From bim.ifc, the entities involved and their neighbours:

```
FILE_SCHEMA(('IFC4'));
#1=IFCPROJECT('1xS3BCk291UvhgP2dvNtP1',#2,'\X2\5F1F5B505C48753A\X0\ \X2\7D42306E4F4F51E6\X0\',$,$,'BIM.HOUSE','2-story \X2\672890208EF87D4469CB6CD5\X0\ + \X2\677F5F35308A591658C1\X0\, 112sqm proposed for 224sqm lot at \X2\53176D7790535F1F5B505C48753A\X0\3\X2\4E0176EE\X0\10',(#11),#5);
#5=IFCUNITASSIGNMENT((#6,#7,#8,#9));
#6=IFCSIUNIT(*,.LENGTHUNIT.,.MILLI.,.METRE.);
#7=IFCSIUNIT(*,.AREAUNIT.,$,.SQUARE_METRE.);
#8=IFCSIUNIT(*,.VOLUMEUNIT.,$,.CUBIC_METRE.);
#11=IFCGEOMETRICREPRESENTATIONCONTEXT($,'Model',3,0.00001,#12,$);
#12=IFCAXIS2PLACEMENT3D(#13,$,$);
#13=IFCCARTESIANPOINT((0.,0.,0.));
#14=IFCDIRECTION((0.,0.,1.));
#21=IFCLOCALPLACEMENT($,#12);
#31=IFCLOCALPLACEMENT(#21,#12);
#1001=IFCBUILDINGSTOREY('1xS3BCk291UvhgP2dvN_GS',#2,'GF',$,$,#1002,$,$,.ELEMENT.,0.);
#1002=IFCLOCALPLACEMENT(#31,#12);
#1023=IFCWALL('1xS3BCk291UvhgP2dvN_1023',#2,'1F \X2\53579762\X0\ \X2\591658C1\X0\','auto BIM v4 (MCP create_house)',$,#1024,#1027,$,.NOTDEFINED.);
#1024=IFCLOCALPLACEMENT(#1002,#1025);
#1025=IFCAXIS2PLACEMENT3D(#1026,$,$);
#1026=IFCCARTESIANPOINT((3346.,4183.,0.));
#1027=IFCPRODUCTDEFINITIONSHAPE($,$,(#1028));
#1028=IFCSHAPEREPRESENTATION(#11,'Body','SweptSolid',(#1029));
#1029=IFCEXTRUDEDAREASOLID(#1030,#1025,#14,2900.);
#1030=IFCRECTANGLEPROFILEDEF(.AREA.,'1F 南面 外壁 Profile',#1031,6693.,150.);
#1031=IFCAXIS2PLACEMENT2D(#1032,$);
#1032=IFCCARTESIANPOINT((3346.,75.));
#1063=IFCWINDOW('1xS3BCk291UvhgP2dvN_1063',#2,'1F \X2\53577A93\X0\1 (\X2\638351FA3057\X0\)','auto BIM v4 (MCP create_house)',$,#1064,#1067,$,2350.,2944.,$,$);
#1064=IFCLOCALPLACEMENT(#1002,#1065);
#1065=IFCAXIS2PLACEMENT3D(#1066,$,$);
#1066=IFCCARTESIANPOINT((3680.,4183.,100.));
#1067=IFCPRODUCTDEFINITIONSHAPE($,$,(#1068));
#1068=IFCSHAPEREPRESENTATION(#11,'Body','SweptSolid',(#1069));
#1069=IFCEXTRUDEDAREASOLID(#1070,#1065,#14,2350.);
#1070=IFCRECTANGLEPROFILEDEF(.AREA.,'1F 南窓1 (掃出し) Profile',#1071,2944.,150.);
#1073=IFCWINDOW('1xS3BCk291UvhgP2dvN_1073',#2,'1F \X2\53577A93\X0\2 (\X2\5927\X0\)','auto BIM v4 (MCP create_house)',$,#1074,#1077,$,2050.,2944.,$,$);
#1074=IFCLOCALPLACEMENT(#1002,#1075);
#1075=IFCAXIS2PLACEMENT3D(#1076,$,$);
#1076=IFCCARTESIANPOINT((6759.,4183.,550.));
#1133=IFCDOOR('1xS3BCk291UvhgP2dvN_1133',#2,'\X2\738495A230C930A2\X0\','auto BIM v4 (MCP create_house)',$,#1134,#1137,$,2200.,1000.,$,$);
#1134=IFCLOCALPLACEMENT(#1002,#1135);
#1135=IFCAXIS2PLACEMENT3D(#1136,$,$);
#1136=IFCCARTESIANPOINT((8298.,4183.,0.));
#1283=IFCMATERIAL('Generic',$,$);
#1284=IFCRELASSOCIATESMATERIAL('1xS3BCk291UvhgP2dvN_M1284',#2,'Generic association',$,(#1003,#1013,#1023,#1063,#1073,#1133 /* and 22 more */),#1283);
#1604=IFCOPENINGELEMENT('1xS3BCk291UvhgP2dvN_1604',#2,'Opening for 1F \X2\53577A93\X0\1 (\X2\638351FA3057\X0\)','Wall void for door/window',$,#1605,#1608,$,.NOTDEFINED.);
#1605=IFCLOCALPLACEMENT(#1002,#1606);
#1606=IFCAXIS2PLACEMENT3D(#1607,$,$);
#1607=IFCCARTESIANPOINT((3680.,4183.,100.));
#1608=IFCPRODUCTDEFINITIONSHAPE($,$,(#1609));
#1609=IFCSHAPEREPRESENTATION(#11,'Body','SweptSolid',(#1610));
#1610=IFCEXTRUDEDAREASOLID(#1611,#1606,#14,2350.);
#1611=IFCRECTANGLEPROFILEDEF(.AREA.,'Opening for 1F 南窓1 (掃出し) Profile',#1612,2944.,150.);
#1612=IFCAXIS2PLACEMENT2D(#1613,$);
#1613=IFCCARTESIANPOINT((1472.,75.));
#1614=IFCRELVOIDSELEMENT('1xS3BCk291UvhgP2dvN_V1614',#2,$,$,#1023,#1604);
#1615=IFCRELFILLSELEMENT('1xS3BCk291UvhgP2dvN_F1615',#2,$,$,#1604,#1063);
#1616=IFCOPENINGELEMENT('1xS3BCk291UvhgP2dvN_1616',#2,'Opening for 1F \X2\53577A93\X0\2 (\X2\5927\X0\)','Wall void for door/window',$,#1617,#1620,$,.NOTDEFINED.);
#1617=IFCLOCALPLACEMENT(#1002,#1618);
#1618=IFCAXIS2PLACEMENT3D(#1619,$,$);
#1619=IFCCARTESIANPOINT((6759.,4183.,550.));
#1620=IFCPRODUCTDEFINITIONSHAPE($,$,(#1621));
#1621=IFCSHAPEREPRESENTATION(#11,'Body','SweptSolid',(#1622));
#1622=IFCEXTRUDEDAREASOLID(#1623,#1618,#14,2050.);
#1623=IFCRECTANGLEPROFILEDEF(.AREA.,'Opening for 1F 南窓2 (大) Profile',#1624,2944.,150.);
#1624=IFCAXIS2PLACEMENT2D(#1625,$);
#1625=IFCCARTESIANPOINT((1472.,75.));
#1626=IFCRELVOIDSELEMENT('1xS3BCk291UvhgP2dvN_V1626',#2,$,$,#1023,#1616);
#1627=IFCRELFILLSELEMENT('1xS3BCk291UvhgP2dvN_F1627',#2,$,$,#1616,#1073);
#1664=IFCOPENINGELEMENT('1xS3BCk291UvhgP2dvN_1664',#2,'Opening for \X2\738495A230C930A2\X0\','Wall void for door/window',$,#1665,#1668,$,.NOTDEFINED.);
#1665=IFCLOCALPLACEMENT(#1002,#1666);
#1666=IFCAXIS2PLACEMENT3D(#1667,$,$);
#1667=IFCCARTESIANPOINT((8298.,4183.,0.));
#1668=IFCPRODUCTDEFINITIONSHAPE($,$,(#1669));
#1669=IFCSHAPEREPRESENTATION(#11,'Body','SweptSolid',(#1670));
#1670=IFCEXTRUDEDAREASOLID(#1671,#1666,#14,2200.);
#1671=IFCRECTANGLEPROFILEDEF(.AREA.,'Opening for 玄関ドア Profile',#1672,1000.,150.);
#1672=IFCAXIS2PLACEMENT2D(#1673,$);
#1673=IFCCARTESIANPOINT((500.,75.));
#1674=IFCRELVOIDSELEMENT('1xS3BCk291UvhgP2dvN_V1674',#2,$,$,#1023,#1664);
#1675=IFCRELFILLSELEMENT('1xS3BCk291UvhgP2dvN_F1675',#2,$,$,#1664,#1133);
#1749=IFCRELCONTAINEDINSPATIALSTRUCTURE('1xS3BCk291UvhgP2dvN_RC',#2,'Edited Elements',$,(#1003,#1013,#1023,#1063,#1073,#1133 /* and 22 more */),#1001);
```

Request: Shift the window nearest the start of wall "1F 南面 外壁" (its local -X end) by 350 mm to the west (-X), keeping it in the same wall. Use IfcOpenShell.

```python
import ifcopenshell
import ifcopenshell.api.geometry
import ifcopenshell.util.placement

model = ifcopenshell.open("bim.ifc")

window = model.by_guid("1xS3BCk291UvhgP2dvN_1063")
opening = window.FillsVoids[0].RelatingOpeningElement
wall = opening.VoidsElements[0].RelatingBuildingElement

wall_matrix = ifcopenshell.util.placement.get_local_placement(wall.ObjectPlacement)
shift = wall_matrix[:3, 0] * -350.0
before = ifcopenshell.util.placement.get_local_placement(window.ObjectPlacement)[:3, 3].copy()

# The window is not placed relative to its opening, so move both.
for product in (opening, window):
    matrix = ifcopenshell.util.placement.get_local_placement(product.ObjectPlacement)
    matrix[:3, 3] += shift
    ifcopenshell.api.geometry.edit_object_placement(model, product=product, matrix=matrix, is_si=False)

after = ifcopenshell.util.placement.get_local_placement(window.ObjectPlacement)[:3, 3]
print("window moved by", (after - before).round(3) + 0.0)

model.write("bim_v2.ifc")
```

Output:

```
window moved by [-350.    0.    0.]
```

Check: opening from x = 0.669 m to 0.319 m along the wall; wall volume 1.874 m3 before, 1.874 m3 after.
